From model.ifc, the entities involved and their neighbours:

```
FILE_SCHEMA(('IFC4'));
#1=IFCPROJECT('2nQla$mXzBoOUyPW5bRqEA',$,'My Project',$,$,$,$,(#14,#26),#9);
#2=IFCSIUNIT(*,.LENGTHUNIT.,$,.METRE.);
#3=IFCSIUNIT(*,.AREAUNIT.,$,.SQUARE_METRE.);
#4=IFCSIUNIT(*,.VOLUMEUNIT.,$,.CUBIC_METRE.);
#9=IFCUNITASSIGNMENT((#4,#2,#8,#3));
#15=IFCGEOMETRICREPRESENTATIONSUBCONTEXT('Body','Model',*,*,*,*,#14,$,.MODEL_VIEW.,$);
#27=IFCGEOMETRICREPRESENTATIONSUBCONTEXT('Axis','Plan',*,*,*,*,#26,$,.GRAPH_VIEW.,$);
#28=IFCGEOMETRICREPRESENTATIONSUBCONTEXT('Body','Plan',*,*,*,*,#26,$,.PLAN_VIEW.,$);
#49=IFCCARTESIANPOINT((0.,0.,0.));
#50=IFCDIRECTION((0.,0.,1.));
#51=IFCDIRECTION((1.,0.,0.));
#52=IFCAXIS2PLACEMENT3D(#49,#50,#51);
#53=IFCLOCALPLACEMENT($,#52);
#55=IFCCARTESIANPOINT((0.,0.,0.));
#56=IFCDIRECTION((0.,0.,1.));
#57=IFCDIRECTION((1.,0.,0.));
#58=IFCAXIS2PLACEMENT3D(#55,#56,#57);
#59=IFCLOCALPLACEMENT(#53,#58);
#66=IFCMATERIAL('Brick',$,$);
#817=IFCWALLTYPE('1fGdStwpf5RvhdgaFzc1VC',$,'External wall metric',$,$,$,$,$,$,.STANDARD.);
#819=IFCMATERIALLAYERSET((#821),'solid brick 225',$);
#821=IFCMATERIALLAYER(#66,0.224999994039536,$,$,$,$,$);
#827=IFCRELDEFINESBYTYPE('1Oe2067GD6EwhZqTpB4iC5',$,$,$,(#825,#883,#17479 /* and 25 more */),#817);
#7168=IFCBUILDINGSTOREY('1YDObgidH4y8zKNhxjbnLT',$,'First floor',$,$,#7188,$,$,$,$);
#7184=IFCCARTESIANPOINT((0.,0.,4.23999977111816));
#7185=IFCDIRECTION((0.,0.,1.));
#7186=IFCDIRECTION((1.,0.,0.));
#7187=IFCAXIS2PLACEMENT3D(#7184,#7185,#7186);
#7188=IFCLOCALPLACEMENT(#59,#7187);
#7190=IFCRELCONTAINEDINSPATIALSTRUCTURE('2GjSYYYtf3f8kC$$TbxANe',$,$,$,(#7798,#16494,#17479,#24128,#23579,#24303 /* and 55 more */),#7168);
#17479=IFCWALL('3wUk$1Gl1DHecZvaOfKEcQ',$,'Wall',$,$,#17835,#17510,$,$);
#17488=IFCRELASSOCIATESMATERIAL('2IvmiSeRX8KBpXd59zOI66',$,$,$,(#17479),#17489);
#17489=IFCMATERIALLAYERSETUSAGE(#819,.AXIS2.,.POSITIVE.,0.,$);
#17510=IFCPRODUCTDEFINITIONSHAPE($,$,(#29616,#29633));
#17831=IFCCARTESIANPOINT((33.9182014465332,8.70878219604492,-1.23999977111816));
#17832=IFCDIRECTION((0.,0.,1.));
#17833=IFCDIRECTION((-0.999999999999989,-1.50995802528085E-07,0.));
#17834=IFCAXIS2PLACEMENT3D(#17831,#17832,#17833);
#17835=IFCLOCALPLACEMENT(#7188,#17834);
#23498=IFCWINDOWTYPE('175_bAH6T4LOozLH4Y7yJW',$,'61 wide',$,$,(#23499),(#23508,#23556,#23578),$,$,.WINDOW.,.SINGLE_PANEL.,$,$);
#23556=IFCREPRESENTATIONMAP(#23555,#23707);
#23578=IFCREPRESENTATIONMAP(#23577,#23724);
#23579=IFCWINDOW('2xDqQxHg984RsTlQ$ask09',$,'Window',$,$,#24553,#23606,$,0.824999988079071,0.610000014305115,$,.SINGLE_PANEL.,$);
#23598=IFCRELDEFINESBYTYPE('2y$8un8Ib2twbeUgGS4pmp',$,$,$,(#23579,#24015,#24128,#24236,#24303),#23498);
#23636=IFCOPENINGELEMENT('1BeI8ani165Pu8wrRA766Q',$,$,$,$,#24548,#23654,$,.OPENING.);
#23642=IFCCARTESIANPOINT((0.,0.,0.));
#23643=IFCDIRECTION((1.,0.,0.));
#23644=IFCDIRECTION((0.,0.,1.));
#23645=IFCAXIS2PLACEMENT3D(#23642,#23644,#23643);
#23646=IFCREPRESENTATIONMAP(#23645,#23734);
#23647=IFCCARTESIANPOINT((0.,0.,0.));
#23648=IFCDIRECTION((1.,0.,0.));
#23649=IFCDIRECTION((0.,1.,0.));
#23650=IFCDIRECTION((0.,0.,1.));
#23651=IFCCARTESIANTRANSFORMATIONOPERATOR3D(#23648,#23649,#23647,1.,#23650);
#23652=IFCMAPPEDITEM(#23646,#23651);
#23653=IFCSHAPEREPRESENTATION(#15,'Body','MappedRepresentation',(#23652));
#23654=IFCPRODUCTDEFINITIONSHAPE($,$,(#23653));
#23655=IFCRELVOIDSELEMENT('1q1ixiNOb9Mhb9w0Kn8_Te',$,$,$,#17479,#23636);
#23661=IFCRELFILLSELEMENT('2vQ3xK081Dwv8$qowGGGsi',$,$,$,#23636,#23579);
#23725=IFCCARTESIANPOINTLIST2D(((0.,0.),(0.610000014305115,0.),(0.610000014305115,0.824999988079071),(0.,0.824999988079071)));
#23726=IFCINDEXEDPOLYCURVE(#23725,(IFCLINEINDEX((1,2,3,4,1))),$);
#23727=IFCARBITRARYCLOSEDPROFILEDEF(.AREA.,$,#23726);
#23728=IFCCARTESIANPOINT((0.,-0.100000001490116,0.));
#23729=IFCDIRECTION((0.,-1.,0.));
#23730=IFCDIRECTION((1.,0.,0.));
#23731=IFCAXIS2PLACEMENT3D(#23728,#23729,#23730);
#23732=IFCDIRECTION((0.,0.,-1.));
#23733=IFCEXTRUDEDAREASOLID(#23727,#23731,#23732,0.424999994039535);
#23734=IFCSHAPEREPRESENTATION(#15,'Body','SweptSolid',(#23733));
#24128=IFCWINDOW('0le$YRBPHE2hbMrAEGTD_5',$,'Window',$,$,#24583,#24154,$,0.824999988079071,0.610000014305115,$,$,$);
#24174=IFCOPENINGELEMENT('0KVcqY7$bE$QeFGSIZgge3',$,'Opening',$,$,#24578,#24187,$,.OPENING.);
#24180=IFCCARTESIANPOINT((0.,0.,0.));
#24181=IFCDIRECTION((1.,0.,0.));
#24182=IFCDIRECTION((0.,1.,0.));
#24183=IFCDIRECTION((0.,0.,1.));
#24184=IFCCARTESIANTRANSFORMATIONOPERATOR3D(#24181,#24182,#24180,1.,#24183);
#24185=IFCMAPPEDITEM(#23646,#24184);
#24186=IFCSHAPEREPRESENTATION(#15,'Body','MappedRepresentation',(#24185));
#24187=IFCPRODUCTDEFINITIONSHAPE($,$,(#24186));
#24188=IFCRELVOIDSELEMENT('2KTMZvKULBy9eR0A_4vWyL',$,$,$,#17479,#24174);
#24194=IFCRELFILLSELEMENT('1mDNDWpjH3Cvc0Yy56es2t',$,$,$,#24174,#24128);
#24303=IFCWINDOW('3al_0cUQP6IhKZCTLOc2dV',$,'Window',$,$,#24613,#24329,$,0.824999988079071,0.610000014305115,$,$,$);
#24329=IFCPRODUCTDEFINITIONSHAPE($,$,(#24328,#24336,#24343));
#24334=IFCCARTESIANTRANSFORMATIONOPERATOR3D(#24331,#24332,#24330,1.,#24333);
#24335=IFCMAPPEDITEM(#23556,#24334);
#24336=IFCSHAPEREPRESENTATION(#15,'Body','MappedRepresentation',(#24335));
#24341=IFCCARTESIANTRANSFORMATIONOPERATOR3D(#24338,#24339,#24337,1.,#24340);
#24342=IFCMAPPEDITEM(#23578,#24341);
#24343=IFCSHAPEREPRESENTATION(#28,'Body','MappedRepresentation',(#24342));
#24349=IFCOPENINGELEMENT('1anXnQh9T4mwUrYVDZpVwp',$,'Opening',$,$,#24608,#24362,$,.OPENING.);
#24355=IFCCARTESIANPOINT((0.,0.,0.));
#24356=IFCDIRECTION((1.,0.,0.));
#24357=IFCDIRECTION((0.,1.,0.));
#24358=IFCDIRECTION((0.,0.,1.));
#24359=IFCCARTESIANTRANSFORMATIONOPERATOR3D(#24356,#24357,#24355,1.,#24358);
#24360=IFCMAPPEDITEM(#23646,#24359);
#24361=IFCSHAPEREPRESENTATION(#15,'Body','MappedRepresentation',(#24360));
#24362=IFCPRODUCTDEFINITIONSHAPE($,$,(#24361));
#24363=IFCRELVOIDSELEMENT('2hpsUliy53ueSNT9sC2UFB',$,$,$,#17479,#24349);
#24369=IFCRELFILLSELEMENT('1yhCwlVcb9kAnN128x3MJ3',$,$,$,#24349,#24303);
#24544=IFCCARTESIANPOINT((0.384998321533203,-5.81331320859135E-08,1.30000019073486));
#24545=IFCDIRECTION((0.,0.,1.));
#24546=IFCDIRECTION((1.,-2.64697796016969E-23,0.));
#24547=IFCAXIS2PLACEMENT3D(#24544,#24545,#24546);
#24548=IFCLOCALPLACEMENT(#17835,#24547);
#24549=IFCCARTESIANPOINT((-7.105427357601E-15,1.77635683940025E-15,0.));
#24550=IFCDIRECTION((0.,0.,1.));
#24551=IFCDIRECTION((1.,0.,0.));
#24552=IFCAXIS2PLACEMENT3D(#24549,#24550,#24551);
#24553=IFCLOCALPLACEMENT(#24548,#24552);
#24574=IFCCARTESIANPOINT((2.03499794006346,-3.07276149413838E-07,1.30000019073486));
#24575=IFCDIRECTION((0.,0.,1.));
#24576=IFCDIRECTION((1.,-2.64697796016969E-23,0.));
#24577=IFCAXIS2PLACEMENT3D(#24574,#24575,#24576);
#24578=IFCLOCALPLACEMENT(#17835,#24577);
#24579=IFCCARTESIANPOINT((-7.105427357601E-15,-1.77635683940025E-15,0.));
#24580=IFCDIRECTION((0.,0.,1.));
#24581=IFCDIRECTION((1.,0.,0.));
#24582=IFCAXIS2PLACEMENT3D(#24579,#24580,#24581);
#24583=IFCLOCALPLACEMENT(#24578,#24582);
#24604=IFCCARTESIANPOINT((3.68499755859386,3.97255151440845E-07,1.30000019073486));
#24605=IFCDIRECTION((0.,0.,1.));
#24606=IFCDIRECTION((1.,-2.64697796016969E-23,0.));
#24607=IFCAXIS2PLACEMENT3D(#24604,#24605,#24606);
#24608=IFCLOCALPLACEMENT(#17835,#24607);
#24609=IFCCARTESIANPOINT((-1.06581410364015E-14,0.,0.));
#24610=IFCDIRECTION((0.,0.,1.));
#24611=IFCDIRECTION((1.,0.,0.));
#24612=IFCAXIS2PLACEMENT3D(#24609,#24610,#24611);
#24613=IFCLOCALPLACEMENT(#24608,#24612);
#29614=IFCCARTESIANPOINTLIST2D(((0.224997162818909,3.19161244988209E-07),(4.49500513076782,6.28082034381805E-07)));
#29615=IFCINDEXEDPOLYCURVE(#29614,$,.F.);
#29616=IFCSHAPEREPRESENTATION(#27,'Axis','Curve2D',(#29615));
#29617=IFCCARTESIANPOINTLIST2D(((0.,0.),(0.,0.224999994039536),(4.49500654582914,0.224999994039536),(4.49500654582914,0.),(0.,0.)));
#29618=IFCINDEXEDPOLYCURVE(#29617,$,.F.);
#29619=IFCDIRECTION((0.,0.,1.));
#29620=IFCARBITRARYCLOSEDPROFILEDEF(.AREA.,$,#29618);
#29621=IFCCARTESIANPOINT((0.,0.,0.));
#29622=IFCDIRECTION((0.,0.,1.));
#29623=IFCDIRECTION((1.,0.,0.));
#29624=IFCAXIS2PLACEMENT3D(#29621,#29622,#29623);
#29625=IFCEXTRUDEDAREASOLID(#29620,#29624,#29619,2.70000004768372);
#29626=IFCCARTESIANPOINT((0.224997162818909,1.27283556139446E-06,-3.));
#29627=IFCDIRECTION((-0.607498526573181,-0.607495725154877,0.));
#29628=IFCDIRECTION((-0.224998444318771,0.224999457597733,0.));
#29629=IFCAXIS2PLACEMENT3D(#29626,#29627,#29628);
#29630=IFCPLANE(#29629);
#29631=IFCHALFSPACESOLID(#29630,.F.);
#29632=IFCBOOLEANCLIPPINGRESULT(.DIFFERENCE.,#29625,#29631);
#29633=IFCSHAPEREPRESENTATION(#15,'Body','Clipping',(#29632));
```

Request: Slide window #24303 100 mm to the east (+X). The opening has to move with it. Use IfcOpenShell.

```python
import ifcopenshell
import ifcopenshell.api.geometry
import ifcopenshell.util.placement
import ifcopenshell.util.unit

model = ifcopenshell.open("model.ifc")
unit_scale = ifcopenshell.util.unit.calculate_unit_scale(model)

window = model.by_id(24303)
opening = window.FillsVoids[0].RelatingOpeningElement
wall = opening.VoidsElements[0].RelatingBuildingElement

wall_matrix = ifcopenshell.util.placement.get_local_placement(wall.ObjectPlacement)
shift = wall_matrix[:3, 0] * -0.1 / unit_scale
before = ifcopenshell.util.placement.get_local_placement(window.ObjectPlacement)[:3, 3].copy()

# The window is placed relative to its opening, so it follows when the opening moves.
matrix = ifcopenshell.util.placement.get_local_placement(opening.ObjectPlacement)
matrix[:3, 3] += shift
ifcopenshell.api.geometry.edit_object_placement(
    model, product=opening, matrix=matrix, is_si=False, should_transform_children=True
)

after = ifcopenshell.util.placement.get_local_placement(window.ObjectPlacement)[:3, 3]
print("window moved by", (after - before).round(3) + 0.0)

model.write("model_updated.ifc")
```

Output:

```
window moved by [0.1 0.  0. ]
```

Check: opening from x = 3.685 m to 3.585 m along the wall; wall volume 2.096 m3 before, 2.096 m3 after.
